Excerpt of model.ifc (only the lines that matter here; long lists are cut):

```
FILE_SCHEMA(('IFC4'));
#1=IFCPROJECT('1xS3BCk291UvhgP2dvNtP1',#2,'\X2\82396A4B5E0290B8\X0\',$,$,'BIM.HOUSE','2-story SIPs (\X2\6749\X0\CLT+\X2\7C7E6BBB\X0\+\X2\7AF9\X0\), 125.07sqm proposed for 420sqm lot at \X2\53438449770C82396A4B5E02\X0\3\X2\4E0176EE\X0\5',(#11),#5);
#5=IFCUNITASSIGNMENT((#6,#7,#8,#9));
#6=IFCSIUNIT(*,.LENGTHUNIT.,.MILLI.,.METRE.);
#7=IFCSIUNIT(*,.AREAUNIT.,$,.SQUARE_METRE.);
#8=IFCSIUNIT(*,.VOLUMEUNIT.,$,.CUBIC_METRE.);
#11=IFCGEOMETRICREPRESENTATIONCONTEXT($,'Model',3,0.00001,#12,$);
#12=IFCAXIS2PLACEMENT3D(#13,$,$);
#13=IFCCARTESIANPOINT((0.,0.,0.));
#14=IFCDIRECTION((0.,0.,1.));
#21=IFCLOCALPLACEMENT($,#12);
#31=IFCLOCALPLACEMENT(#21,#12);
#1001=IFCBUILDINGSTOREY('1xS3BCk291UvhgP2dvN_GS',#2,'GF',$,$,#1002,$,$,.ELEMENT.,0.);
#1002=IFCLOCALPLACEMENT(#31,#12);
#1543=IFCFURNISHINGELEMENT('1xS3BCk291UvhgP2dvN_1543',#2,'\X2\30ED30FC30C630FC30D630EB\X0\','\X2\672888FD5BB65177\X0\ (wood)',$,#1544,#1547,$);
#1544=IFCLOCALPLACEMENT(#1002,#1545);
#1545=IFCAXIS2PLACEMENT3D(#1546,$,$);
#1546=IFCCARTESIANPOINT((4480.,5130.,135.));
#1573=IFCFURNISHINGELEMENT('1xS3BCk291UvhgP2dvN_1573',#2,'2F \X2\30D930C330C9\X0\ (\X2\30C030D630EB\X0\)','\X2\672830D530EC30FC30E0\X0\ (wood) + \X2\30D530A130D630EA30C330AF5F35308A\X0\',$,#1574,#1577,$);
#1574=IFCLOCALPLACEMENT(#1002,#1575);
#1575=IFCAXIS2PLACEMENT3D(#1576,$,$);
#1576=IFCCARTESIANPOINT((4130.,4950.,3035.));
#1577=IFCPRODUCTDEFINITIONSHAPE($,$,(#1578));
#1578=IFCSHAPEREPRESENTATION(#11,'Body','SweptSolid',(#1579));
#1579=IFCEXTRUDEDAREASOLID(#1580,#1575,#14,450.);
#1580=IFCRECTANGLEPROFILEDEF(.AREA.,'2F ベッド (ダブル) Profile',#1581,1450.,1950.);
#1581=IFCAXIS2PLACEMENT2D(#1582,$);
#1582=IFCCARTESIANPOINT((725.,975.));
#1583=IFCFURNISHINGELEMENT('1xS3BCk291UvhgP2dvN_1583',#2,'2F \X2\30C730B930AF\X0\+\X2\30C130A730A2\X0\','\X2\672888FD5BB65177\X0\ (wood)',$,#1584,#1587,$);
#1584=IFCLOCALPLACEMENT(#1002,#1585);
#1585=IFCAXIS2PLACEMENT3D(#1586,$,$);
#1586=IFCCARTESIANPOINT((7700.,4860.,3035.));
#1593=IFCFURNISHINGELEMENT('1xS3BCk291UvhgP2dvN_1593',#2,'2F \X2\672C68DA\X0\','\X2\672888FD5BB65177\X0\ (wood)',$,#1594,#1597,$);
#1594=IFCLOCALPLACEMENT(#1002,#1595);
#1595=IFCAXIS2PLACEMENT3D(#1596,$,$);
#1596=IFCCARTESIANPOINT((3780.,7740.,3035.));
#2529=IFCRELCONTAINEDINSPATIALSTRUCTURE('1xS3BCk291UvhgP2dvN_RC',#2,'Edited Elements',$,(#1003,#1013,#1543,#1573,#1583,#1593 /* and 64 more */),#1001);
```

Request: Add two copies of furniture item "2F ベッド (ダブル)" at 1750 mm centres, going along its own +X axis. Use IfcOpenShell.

```python
import ifcopenshell
import ifcopenshell.api.geometry
import ifcopenshell.api.root
import ifcopenshell.util.element
import ifcopenshell.util.placement

model = ifcopenshell.open("model.ifc")


def reuse_history(source, copy):
    """copy_class also copies each property set's owner history, people and application; keep the originals."""
    for rel in copy.IsDefinedBy:
        if rel.is_a("IfcRelDefinesByProperties") and (history := rel.RelatingPropertyDefinition.OwnerHistory):
            rel.RelatingPropertyDefinition.OwnerHistory = source.OwnerHistory
            ifcopenshell.util.element.remove_deep2(model, history)


source = model.by_guid("1xS3BCk291UvhgP2dvN_1573")
base = ifcopenshell.util.placement.get_local_placement(source.ObjectPlacement)
step = base[:3, 0] * 1750.0

for i in range(1, 3):
    copy = ifcopenshell.api.root.copy_class(model, product=source)
    copy.Representation = ifcopenshell.util.element.copy_deep(
        model, source.Representation, exclude=["IfcGeometricRepresentationContext", "IfcRepresentationMap"]
    )
    reuse_history(source, copy)
    matrix = base.copy()
    matrix[:3, 3] += i * step
    print("added at", matrix[:3, 3].round(3) + 0.0)
    ifcopenshell.api.geometry.edit_object_placement(model, product=copy, matrix=matrix, is_si=False)

model.write("model_updated.ifc")
```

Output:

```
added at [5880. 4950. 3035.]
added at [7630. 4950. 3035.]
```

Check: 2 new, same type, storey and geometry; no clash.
